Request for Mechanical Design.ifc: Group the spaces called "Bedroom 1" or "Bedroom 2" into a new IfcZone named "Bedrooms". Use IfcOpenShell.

First a look at what the model holds.

```python
import ifcopenshell

model = ifcopenshell.open("Mechanical Design.ifc")
print(model.schema)
seen = {}
for space in model.by_type("IfcSpace"):
    seen[space.LongName] = seen.get(space.LongName, 0) + 1
for name, count in sorted(seen.items(), key=str):
    print(count, "x", name)
print("zones:", [z.Name for z in model.by_type("IfcZone")][:20])
```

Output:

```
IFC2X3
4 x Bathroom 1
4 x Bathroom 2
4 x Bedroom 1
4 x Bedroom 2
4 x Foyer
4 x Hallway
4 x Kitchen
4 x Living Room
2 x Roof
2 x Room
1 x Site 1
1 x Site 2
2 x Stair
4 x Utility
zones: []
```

```python
import ifcopenshell
import ifcopenshell.api.group
import ifcopenshell.api.root

model = ifcopenshell.open("Mechanical Design.ifc")

names = {"Bedroom 1", "Bedroom 2"}
spaces = [s for s in model.by_type("IfcSpace") if s.LongName in names]

zone = ifcopenshell.api.root.create_entity(model, ifc_class="IfcZone", name="Bedrooms")
ifcopenshell.api.group.assign_group(model, products=spaces, group=zone)
print(len(spaces), "spaces in", zone.Name)

model.write("Mechanical Design-out.ifc")
```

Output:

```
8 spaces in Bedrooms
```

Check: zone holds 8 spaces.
